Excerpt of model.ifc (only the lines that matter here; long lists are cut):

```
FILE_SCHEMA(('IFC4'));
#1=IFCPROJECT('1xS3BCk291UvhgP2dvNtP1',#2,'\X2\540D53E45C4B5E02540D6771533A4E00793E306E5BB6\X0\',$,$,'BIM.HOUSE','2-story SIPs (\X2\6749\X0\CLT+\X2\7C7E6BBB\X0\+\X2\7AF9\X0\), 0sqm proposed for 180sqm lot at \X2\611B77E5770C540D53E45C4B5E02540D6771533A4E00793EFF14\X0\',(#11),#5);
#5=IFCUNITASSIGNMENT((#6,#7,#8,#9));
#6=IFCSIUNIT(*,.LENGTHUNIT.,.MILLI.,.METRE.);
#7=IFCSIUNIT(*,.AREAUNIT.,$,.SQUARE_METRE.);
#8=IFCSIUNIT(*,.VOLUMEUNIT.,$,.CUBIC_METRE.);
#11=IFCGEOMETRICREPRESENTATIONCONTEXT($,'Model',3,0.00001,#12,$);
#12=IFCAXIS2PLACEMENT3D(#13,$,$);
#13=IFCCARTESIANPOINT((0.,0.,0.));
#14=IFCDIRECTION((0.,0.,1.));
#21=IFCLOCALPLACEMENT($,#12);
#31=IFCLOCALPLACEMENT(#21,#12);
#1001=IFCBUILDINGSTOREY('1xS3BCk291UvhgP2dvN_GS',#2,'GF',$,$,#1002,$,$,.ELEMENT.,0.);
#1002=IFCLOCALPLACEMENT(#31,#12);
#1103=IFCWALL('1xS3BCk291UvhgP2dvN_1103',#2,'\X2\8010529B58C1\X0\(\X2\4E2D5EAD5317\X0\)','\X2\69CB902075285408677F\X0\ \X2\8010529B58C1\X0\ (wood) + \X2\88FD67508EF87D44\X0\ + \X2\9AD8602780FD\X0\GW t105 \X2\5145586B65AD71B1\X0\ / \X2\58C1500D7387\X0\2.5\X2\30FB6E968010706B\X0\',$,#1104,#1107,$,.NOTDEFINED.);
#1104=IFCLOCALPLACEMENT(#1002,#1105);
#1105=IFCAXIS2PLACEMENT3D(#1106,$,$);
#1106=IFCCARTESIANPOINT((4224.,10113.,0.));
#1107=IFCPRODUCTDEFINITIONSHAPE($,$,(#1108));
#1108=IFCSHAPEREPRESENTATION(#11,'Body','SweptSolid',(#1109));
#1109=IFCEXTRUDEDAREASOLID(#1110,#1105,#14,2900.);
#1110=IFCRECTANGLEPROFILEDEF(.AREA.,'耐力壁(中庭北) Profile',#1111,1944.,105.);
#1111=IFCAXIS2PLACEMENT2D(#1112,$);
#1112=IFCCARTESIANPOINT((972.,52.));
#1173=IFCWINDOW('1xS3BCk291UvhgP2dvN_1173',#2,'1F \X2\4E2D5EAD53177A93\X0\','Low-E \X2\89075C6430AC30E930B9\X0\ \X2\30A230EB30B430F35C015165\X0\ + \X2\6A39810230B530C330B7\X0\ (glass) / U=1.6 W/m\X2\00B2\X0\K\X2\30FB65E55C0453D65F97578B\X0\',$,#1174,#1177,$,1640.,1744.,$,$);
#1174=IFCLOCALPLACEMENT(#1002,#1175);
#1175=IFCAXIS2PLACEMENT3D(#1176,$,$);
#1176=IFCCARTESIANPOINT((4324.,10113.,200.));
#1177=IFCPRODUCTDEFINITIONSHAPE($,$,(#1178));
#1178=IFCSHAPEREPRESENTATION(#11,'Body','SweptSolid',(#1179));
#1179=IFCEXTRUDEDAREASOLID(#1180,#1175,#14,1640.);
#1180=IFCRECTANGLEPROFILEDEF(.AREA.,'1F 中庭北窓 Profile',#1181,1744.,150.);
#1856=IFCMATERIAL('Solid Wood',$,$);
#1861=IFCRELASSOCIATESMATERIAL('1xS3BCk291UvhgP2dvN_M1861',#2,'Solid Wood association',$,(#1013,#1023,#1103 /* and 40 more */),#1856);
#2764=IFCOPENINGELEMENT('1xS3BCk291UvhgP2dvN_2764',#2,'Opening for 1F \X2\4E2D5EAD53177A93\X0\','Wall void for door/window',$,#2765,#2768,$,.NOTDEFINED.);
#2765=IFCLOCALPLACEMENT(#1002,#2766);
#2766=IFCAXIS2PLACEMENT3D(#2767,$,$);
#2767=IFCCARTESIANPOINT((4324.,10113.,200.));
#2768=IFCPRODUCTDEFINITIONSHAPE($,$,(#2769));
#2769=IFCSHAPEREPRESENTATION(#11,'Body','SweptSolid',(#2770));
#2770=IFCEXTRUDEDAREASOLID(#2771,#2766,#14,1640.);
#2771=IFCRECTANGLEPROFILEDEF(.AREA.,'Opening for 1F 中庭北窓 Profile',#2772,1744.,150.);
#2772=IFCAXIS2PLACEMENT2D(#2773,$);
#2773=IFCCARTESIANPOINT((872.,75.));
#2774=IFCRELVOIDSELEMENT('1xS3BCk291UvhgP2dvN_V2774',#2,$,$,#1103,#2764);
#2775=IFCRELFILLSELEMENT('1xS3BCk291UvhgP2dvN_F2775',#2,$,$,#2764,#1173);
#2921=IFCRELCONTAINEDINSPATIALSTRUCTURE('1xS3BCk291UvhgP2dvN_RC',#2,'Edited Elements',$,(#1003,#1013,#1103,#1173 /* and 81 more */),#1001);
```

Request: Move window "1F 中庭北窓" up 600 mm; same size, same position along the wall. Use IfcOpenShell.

```python
import numpy as np
import ifcopenshell
import ifcopenshell.api.geometry
import ifcopenshell.util.placement
import ifcopenshell.util.unit

model = ifcopenshell.open("model.ifc")
unit_scale = ifcopenshell.util.unit.calculate_unit_scale(model)

window = model.by_id(1173)
opening = window.FillsVoids[0].RelatingOpeningElement
dz = 0.6 / unit_scale

shift = np.array([0.0, 0.0, dz])
# The window is not placed relative to its opening, so move both.
for product in (opening, window):
    matrix = ifcopenshell.util.placement.get_local_placement(product.ObjectPlacement)
    matrix[:3, 3] += shift
    ifcopenshell.api.geometry.edit_object_placement(model, product=product, matrix=matrix, is_si=False)

print(f"moved by {dz * unit_scale:+.3f} m")

model.write("model_updated.ifc")
```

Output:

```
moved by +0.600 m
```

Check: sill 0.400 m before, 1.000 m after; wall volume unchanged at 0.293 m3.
